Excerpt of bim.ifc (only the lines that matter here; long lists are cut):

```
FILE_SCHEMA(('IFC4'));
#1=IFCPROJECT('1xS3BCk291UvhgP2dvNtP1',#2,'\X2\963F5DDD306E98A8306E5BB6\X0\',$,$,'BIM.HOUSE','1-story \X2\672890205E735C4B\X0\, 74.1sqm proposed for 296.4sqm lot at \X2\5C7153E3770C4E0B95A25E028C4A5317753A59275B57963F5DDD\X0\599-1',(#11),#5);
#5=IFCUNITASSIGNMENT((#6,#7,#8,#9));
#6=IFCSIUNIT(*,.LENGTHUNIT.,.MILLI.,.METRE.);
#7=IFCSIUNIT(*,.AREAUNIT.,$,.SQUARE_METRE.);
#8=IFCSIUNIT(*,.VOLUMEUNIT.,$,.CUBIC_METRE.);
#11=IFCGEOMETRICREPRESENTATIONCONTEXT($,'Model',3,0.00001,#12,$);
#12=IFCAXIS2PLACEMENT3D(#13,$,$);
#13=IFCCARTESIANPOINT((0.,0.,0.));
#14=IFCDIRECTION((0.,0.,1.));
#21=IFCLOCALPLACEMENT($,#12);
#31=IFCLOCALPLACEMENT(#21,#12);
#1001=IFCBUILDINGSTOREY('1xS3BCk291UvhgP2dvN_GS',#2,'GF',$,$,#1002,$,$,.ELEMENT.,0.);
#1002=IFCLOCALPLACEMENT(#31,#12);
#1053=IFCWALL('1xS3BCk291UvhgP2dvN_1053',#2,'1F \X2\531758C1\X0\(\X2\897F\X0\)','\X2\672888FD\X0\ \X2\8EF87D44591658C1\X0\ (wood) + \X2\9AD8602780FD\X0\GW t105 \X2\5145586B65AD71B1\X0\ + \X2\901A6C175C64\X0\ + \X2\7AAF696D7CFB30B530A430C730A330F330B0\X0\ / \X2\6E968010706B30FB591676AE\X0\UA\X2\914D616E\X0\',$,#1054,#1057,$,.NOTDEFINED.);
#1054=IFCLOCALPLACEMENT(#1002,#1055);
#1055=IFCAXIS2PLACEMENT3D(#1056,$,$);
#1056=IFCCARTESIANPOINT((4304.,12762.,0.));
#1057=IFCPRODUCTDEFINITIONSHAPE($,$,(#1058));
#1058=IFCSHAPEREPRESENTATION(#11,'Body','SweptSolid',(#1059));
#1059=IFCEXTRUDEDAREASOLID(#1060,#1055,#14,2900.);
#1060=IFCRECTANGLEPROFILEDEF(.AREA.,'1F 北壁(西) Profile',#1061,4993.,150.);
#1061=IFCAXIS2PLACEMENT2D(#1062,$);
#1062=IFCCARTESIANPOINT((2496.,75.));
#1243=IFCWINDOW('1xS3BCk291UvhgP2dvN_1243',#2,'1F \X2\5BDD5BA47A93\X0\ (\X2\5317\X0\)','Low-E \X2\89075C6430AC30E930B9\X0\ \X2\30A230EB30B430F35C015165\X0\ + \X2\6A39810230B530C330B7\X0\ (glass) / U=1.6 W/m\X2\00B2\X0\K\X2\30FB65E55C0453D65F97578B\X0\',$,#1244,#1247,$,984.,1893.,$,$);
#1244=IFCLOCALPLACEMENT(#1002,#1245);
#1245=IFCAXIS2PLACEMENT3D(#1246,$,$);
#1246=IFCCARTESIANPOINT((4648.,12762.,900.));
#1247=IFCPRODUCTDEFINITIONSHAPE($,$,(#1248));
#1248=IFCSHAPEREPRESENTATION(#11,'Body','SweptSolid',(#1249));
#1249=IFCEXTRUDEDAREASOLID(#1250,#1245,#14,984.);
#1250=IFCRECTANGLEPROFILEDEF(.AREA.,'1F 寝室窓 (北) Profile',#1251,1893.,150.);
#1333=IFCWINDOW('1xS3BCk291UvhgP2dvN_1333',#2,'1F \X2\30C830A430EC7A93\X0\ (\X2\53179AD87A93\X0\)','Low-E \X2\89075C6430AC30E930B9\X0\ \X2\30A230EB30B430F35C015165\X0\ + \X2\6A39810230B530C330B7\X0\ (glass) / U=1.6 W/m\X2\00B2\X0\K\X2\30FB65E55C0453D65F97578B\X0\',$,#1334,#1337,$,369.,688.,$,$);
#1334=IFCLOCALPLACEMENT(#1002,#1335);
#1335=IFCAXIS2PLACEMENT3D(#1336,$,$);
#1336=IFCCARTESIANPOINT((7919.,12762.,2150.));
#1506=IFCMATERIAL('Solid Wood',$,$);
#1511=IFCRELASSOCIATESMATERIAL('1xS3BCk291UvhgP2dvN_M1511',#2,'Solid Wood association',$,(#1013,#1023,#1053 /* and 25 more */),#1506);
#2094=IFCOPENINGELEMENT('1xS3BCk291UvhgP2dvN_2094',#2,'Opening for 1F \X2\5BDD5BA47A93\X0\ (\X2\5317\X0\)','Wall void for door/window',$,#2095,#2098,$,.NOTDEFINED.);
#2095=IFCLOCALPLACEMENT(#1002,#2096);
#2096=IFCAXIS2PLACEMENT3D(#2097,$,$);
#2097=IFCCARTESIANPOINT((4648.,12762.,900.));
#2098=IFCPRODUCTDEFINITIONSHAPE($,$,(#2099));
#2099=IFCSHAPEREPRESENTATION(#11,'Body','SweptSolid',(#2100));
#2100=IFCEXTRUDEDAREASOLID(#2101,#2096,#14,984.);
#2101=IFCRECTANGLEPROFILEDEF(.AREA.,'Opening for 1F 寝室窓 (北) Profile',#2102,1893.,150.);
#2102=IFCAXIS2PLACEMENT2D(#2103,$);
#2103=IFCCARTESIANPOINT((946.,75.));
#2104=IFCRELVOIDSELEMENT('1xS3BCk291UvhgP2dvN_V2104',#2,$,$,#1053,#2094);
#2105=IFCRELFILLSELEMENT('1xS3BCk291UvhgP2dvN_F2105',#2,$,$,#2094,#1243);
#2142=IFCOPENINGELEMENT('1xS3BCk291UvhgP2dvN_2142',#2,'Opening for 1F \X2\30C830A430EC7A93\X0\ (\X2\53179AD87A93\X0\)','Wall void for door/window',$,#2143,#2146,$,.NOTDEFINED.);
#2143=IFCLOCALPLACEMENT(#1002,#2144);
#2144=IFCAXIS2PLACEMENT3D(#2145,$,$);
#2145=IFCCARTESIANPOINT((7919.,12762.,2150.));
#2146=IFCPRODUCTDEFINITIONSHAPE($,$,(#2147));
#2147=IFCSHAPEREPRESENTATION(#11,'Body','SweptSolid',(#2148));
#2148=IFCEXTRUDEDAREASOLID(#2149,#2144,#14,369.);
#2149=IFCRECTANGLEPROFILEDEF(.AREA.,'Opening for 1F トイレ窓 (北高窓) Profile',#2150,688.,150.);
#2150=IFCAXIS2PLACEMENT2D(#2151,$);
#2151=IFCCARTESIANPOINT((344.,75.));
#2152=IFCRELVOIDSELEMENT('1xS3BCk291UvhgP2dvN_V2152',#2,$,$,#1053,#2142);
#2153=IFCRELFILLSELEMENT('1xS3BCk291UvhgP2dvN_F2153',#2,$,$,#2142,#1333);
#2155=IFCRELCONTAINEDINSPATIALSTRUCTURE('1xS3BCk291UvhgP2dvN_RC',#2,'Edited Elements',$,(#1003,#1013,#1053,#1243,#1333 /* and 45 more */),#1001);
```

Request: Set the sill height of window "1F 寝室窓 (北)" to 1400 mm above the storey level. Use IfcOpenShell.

```python
import numpy as np
import ifcopenshell
import ifcopenshell.api.geometry
import ifcopenshell.geom
import ifcopenshell.util.element
import ifcopenshell.util.placement
import ifcopenshell.util.shape
import ifcopenshell.util.unit

model = ifcopenshell.open("bim.ifc")
unit_scale = ifcopenshell.util.unit.calculate_unit_scale(model)

window = model.by_guid("1xS3BCk291UvhgP2dvN_1243")
opening = window.FillsVoids[0].RelatingOpeningElement
storey = ifcopenshell.util.element.get_container(window, ifc_class="IfcBuildingStorey")
level = ifcopenshell.util.placement.get_local_placement(storey.ObjectPlacement)[2, 3]

# The opening's origin need not be at the sill, so measure its lowest point.
shape = ifcopenshell.geom.create_shape(ifcopenshell.geom.settings(), opening)
bottom = ifcopenshell.util.shape.get_shape_bottom_elevation(shape, shape.geometry) / unit_scale
dz = level + 1400.0 - bottom

shift = np.array([0.0, 0.0, dz])
# The window is not placed relative to its opening, so move both.
for product in (opening, window):
    matrix = ifcopenshell.util.placement.get_local_placement(product.ObjectPlacement)
    matrix[:3, 3] += shift
    ifcopenshell.api.geometry.edit_object_placement(model, product=product, matrix=matrix, is_si=False)

print(f"moved by {dz * unit_scale:+.3f} m")

model.write("bim_edited.ifc")
```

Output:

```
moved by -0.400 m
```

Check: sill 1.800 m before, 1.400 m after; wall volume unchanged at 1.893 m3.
